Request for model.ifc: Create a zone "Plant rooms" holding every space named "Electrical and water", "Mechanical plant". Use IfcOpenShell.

First a look at what the model holds.

```python
import ifcopenshell

model = ifcopenshell.open("model.ifc")
print(model.schema)
seen = {}
for space in model.by_type("IfcSpace"):
    seen[space.LongName] = seen.get(space.LongName, 0) + 1
for name, count in sorted(seen.items(), key=str):
    print(count, "x", name)
print("zones:", [z.Name for z in model.by_type("IfcZone")][:20])
```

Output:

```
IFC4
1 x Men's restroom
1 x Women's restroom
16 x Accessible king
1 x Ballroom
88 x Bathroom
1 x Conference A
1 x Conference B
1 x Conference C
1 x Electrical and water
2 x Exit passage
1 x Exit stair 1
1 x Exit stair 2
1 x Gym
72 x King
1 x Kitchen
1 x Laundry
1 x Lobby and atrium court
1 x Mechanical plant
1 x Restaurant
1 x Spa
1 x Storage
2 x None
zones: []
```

```python
import ifcopenshell
import ifcopenshell.api.group
import ifcopenshell.api.root

model = ifcopenshell.open("model.ifc")

names = {"Electrical and water", "Mechanical plant"}
spaces = [s for s in model.by_type("IfcSpace") if s.LongName in names]

zone = ifcopenshell.api.root.create_entity(model, ifc_class="IfcZone", name="Plant rooms")
ifcopenshell.api.group.assign_group(model, products=spaces, group=zone)
print(len(spaces), "spaces in", zone.Name)

model.write("model_v2.ifc")
```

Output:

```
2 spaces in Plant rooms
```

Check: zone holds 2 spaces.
